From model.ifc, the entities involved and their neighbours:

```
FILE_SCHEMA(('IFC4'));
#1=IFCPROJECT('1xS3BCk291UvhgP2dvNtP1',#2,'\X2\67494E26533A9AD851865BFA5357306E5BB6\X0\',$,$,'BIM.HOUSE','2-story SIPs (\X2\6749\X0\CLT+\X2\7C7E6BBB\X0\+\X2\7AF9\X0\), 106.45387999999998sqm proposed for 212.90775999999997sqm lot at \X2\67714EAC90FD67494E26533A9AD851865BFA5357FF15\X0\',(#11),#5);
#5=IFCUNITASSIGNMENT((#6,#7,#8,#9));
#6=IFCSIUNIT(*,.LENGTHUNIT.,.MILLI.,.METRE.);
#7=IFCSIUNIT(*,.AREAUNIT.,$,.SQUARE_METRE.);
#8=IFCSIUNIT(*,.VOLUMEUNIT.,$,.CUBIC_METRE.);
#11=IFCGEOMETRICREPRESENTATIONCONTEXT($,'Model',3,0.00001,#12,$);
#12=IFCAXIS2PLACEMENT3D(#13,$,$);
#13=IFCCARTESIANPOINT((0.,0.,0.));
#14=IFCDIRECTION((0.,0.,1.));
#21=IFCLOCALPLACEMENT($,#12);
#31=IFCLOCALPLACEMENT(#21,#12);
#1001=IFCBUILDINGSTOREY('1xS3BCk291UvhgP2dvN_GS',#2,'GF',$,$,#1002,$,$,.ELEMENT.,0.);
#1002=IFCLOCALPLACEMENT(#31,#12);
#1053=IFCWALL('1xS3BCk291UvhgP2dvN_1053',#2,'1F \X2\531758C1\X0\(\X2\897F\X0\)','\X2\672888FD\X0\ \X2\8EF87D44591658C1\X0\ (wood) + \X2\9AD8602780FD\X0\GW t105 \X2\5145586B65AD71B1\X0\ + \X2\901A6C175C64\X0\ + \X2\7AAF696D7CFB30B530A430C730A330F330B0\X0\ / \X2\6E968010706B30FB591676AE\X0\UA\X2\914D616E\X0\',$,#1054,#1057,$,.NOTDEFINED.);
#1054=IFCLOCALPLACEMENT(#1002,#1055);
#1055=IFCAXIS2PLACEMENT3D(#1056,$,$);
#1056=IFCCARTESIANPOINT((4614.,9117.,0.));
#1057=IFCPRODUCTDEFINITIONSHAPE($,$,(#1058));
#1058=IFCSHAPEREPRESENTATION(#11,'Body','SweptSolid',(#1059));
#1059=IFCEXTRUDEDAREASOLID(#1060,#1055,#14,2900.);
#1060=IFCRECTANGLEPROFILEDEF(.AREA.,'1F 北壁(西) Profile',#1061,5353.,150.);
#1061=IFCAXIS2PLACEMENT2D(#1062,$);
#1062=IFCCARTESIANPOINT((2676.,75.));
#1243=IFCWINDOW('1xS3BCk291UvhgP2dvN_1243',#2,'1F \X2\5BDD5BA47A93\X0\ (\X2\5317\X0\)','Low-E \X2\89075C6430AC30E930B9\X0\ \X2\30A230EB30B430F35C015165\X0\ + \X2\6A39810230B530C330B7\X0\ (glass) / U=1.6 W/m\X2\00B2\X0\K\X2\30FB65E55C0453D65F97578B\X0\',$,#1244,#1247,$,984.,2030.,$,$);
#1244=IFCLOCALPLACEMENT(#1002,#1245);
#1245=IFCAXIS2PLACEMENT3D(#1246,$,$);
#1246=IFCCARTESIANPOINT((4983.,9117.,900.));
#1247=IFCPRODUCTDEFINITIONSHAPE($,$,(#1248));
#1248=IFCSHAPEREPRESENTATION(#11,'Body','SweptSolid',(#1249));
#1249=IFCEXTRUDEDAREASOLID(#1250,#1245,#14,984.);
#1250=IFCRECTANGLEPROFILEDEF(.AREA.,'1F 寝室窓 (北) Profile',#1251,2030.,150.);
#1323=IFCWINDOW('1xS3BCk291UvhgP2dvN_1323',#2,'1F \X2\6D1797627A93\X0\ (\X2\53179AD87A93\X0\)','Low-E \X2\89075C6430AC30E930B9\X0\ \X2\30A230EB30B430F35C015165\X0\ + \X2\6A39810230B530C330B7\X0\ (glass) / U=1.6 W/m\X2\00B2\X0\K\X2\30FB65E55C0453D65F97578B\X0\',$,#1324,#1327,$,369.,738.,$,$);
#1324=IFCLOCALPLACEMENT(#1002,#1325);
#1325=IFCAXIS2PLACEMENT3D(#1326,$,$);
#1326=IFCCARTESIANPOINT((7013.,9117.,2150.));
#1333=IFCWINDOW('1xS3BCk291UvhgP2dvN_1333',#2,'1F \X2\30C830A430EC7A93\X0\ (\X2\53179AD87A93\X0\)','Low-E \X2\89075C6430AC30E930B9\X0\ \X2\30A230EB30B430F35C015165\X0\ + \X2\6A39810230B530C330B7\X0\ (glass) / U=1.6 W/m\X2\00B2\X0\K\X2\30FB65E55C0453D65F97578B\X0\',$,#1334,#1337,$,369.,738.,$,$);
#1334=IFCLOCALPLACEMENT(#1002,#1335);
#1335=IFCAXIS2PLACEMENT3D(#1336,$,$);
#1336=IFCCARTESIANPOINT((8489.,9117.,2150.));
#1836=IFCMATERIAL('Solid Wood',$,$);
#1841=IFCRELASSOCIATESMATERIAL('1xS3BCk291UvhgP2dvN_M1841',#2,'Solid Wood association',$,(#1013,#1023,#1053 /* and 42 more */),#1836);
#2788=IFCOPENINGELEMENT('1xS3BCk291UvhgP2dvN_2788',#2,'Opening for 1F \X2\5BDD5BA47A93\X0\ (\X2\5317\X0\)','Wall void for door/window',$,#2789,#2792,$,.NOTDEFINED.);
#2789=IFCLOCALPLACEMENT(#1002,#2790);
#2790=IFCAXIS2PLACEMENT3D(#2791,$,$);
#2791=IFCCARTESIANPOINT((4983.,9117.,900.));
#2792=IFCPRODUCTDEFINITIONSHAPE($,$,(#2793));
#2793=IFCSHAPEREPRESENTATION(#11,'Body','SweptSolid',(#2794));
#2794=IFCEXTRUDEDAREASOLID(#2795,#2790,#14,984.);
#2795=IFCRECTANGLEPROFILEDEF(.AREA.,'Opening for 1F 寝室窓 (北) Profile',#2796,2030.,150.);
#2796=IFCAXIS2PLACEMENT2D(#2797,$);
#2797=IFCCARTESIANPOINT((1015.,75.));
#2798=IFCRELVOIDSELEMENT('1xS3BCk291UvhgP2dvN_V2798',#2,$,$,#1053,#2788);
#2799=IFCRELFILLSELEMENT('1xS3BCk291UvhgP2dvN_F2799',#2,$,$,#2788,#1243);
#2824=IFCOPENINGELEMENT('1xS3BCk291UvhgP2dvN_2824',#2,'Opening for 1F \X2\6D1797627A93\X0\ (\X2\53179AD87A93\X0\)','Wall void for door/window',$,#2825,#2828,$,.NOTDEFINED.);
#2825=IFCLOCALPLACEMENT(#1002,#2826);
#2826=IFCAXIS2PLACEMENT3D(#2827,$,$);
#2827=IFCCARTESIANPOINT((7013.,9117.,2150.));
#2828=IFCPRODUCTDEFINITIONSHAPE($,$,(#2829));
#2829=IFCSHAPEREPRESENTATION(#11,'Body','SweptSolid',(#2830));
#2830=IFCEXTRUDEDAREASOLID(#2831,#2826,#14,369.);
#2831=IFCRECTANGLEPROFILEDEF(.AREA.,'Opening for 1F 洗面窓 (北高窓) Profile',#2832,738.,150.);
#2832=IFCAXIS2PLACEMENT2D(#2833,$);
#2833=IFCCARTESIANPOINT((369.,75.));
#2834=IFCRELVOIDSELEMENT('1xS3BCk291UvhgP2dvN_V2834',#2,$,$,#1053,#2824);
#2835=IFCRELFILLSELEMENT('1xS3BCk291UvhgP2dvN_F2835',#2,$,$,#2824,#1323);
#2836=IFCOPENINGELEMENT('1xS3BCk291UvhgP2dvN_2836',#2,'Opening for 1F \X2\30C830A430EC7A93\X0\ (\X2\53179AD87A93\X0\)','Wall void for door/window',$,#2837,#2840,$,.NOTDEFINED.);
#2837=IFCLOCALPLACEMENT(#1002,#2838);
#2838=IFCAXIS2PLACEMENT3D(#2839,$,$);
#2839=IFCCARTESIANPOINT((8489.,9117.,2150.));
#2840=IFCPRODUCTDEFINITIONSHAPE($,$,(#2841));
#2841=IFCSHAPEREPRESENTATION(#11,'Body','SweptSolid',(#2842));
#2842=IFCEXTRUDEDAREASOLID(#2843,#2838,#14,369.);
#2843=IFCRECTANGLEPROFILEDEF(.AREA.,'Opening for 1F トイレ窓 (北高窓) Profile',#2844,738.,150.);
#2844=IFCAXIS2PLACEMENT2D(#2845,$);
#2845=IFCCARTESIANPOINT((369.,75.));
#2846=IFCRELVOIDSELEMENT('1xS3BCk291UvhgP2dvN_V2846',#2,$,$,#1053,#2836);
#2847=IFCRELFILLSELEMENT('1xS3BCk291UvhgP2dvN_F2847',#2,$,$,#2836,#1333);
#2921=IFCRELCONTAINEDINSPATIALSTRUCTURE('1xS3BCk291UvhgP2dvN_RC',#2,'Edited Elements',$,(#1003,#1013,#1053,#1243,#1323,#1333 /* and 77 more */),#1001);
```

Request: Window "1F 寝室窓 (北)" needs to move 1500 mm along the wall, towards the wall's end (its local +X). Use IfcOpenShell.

```python
import ifcopenshell
import ifcopenshell.api.geometry
import ifcopenshell.util.placement
import ifcopenshell.util.unit

model = ifcopenshell.open("model.ifc")
unit_scale = ifcopenshell.util.unit.calculate_unit_scale(model)

window = model.by_id(1243)
opening = window.FillsVoids[0].RelatingOpeningElement
wall = opening.VoidsElements[0].RelatingBuildingElement

wall_matrix = ifcopenshell.util.placement.get_local_placement(wall.ObjectPlacement)
shift = wall_matrix[:3, 0] * 1.5 / unit_scale
before = ifcopenshell.util.placement.get_local_placement(window.ObjectPlacement)[:3, 3].copy()

# The window is not placed relative to its opening, so move both.
for product in (opening, window):
    matrix = ifcopenshell.util.placement.get_local_placement(product.ObjectPlacement)
    matrix[:3, 3] += shift
    ifcopenshell.api.geometry.edit_object_placement(model, product=product, matrix=matrix, is_si=False)

after = ifcopenshell.util.placement.get_local_placement(window.ObjectPlacement)[:3, 3]
print("window moved by", (after - before).round(3) + 0.0)

model.write("model_v2.ifc")
```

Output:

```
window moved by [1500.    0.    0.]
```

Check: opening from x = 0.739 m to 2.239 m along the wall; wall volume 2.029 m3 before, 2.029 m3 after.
